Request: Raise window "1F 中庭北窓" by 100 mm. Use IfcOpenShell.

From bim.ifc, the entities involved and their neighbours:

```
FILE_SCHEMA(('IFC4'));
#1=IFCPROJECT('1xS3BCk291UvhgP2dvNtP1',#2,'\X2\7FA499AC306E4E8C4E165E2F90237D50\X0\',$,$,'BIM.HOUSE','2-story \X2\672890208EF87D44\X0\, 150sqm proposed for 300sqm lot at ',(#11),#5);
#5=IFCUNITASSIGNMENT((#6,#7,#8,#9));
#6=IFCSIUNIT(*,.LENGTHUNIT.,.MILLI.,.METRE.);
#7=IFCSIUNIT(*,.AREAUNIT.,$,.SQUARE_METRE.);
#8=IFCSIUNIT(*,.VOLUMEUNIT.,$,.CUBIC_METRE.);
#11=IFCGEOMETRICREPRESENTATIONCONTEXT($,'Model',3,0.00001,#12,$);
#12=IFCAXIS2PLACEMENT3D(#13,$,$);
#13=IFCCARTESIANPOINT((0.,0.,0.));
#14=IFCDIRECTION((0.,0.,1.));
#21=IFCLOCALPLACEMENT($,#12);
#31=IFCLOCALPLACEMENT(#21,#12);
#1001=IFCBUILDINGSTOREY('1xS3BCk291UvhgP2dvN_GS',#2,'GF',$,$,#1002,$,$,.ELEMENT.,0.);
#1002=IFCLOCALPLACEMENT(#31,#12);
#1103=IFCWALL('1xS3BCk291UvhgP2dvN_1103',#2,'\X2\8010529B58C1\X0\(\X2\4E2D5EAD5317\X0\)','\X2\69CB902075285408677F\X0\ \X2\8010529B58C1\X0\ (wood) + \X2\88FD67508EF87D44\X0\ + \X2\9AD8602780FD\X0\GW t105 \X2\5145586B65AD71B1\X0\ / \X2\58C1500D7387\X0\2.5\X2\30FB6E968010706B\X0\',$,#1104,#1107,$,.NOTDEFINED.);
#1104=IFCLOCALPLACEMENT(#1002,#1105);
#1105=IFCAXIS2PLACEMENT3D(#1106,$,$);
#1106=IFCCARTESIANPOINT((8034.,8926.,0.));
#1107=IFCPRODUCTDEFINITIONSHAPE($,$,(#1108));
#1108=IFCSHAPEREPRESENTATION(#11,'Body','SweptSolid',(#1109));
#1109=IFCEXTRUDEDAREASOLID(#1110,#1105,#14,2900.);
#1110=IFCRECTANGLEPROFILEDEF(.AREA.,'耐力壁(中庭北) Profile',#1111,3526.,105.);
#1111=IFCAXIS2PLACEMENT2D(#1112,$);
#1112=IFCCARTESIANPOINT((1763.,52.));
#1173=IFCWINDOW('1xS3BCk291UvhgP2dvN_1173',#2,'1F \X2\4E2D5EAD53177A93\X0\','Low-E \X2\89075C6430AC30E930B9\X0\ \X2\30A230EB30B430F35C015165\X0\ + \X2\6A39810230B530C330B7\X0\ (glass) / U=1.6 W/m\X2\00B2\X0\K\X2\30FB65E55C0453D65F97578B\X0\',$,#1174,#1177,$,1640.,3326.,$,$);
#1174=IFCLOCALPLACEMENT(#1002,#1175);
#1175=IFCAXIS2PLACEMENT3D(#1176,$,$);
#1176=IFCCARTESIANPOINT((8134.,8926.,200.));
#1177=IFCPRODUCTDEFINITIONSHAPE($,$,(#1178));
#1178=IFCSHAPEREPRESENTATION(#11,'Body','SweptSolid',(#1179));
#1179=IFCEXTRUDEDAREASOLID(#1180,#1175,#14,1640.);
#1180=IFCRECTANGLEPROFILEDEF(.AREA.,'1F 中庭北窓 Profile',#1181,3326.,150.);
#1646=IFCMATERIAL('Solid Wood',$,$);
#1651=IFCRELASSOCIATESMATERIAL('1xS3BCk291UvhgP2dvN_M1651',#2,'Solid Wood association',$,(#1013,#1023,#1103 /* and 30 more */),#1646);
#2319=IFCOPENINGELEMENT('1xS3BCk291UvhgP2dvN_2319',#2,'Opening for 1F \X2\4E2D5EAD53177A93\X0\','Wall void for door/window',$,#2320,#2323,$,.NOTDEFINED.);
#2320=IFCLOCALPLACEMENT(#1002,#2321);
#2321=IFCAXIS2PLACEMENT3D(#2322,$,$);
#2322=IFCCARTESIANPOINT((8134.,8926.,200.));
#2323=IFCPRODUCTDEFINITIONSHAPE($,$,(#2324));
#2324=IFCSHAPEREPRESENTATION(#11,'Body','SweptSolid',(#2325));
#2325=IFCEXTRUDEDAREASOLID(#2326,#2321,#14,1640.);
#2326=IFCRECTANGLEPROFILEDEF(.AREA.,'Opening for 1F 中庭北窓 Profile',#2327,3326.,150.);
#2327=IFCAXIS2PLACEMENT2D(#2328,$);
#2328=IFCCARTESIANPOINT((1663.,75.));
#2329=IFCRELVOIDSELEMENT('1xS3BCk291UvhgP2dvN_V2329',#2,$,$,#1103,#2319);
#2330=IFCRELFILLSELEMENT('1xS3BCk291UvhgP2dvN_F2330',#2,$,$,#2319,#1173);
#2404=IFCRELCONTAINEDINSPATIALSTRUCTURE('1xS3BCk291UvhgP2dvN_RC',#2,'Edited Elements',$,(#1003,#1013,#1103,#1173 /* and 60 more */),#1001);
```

```python
import numpy as np
import ifcopenshell
import ifcopenshell.api.geometry
import ifcopenshell.util.placement
import ifcopenshell.util.unit

model = ifcopenshell.open("bim.ifc")
unit_scale = ifcopenshell.util.unit.calculate_unit_scale(model)

window = model.by_guid("1xS3BCk291UvhgP2dvN_1173")
opening = window.FillsVoids[0].RelatingOpeningElement
dz = 100.0

shift = np.array([0.0, 0.0, dz])
# The window is not placed relative to its opening, so move both.
for product in (opening, window):
    matrix = ifcopenshell.util.placement.get_local_placement(product.ObjectPlacement)
    matrix[:3, 3] += shift
    ifcopenshell.api.geometry.edit_object_placement(model, product=product, matrix=matrix, is_si=False)

print(f"moved by {dz * unit_scale:+.3f} m")

model.write("bim-out.ifc")
```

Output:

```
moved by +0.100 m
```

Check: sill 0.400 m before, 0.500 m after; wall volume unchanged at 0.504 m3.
